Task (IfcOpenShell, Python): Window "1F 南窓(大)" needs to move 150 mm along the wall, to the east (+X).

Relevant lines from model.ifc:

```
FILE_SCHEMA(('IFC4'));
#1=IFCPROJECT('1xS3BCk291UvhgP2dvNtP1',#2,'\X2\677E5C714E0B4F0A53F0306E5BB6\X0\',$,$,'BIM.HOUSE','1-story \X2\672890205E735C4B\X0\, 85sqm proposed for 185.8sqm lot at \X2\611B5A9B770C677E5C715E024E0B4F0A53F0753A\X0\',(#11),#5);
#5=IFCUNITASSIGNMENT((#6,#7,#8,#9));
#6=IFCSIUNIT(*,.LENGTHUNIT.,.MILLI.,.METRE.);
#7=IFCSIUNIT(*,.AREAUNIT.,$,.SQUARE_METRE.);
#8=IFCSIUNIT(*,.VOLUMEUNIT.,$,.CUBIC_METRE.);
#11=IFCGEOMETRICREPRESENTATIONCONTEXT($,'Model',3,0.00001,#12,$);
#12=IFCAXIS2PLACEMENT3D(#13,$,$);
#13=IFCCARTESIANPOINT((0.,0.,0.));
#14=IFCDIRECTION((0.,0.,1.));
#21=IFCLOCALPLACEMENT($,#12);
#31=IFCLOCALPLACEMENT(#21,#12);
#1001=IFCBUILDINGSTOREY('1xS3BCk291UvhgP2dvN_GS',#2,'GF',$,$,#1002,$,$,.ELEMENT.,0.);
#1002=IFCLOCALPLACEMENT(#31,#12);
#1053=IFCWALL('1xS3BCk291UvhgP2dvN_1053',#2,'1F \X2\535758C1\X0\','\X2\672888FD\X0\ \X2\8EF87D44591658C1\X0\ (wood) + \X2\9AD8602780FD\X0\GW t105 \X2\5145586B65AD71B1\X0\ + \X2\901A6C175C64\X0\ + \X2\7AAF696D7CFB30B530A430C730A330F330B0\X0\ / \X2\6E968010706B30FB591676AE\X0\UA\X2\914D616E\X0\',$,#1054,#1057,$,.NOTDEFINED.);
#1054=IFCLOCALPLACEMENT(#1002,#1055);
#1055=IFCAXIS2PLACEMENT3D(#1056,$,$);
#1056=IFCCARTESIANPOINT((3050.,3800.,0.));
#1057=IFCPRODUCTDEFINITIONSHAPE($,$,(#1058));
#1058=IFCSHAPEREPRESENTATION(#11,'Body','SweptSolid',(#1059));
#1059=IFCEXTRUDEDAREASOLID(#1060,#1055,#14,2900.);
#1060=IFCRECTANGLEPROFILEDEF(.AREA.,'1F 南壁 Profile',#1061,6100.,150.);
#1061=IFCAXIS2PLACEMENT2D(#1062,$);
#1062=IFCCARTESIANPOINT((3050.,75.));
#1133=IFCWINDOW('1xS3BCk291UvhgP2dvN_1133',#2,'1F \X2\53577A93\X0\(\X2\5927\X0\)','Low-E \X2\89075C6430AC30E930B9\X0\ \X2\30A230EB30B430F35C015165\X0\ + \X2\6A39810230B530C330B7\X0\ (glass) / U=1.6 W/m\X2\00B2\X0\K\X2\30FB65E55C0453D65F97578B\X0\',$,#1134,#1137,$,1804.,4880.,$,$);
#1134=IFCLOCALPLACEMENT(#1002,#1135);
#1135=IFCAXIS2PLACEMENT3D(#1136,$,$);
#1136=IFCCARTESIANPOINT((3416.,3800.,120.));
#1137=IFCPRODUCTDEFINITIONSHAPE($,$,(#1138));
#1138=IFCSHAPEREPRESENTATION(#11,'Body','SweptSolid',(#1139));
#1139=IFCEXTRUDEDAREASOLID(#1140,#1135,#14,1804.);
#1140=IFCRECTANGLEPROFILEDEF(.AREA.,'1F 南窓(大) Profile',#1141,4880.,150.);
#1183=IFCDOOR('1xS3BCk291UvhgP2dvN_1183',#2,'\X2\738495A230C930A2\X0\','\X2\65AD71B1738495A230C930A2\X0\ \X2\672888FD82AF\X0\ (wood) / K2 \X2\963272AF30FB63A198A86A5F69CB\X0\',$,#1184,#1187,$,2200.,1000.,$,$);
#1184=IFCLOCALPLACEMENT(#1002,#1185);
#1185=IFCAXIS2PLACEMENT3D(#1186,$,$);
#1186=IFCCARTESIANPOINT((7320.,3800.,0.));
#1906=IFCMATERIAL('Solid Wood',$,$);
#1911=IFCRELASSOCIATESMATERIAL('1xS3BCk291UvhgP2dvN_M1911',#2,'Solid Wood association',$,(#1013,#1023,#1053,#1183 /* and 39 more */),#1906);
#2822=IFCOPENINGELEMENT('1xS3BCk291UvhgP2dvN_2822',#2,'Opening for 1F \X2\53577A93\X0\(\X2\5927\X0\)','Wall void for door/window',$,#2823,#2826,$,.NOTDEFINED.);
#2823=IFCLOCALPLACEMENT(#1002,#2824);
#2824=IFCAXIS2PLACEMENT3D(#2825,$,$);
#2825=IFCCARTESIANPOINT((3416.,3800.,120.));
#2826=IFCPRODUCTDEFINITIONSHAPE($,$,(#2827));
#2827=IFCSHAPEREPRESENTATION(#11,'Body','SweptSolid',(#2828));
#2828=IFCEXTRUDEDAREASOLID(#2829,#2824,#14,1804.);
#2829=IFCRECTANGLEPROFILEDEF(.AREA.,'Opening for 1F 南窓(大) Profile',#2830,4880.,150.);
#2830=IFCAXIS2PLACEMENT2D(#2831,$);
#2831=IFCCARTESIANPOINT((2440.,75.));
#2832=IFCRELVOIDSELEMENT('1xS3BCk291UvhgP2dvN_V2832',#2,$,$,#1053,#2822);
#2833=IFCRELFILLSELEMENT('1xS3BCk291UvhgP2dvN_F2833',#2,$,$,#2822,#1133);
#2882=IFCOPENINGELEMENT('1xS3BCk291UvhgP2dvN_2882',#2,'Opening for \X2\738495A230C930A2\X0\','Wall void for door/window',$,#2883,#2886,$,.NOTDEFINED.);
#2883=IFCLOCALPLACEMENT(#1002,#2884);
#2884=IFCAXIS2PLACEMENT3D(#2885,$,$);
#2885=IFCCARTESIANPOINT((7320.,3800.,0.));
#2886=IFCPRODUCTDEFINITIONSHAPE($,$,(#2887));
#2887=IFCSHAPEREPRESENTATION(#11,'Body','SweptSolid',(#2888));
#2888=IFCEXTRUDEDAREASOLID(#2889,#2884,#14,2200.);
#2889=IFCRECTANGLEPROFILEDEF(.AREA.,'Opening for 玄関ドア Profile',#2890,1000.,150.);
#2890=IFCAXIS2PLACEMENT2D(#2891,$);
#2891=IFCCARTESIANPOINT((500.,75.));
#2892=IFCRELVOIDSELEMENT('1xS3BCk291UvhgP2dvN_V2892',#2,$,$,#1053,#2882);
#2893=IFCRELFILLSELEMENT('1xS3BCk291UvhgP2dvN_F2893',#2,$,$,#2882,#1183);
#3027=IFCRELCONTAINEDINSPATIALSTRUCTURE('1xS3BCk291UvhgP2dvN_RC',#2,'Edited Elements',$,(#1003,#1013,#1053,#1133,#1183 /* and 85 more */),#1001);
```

```python
import ifcopenshell
import ifcopenshell.api.geometry
import ifcopenshell.util.placement
import ifcopenshell.util.unit

model = ifcopenshell.open("model.ifc")
unit_scale = ifcopenshell.util.unit.calculate_unit_scale(model)

window = model.by_id(1133)
opening = window.FillsVoids[0].RelatingOpeningElement
wall = opening.VoidsElements[0].RelatingBuildingElement

wall_matrix = ifcopenshell.util.placement.get_local_placement(wall.ObjectPlacement)
shift = wall_matrix[:3, 0] * 0.15 / unit_scale
before = ifcopenshell.util.placement.get_local_placement(window.ObjectPlacement)[:3, 3].copy()

# The window is not placed relative to its opening, so move both.
for product in (opening, window):
    matrix = ifcopenshell.util.placement.get_local_placement(product.ObjectPlacement)
    matrix[:3, 3] += shift
    ifcopenshell.api.geometry.edit_object_placement(model, product=product, matrix=matrix, is_si=False)

after = ifcopenshell.util.placement.get_local_placement(window.ObjectPlacement)[:3, 3]
print("window moved by", (after - before).round(3) + 0.0)

model.write("model-out.ifc")
```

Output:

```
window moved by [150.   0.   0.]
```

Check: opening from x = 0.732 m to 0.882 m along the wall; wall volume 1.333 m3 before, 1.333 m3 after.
